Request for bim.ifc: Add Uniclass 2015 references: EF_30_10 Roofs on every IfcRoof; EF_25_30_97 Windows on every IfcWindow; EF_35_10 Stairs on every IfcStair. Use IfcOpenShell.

First a look at what the model holds.

```python
import ifcopenshell

model = ifcopenshell.open("bim.ifc")
print(model.schema)
print("classifications:", [c.Name for c in model.by_type("IfcClassification")])
for ifc_class in ("IfcDoor", "IfcRoof", "IfcStair", "IfcWall", "IfcWindow"):
    print(ifc_class, len(model.by_type(ifc_class)))
```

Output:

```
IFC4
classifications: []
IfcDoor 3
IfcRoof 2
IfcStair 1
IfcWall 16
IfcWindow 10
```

```python
import ifcopenshell
import ifcopenshell.api.classification

model = ifcopenshell.open("bim.ifc")

system = ifcopenshell.api.classification.add_classification(model, classification="Uniclass 2015")

codes = {
    "IfcRoof": ("EF_30_10", "Roofs"),
    "IfcWindow": ("EF_25_30_97", "Windows"),
    "IfcStair": ("EF_35_10", "Stairs"),
}
for ifc_class, (code, name) in codes.items():
    products = model.by_type(ifc_class)
    ifcopenshell.api.classification.add_reference(
        model, products=products, classification=system, identification=code, name=name
    )
    print(code, len(products))

model.write("bim_v2.ifc")
```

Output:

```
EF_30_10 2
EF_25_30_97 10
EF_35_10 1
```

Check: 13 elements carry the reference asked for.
